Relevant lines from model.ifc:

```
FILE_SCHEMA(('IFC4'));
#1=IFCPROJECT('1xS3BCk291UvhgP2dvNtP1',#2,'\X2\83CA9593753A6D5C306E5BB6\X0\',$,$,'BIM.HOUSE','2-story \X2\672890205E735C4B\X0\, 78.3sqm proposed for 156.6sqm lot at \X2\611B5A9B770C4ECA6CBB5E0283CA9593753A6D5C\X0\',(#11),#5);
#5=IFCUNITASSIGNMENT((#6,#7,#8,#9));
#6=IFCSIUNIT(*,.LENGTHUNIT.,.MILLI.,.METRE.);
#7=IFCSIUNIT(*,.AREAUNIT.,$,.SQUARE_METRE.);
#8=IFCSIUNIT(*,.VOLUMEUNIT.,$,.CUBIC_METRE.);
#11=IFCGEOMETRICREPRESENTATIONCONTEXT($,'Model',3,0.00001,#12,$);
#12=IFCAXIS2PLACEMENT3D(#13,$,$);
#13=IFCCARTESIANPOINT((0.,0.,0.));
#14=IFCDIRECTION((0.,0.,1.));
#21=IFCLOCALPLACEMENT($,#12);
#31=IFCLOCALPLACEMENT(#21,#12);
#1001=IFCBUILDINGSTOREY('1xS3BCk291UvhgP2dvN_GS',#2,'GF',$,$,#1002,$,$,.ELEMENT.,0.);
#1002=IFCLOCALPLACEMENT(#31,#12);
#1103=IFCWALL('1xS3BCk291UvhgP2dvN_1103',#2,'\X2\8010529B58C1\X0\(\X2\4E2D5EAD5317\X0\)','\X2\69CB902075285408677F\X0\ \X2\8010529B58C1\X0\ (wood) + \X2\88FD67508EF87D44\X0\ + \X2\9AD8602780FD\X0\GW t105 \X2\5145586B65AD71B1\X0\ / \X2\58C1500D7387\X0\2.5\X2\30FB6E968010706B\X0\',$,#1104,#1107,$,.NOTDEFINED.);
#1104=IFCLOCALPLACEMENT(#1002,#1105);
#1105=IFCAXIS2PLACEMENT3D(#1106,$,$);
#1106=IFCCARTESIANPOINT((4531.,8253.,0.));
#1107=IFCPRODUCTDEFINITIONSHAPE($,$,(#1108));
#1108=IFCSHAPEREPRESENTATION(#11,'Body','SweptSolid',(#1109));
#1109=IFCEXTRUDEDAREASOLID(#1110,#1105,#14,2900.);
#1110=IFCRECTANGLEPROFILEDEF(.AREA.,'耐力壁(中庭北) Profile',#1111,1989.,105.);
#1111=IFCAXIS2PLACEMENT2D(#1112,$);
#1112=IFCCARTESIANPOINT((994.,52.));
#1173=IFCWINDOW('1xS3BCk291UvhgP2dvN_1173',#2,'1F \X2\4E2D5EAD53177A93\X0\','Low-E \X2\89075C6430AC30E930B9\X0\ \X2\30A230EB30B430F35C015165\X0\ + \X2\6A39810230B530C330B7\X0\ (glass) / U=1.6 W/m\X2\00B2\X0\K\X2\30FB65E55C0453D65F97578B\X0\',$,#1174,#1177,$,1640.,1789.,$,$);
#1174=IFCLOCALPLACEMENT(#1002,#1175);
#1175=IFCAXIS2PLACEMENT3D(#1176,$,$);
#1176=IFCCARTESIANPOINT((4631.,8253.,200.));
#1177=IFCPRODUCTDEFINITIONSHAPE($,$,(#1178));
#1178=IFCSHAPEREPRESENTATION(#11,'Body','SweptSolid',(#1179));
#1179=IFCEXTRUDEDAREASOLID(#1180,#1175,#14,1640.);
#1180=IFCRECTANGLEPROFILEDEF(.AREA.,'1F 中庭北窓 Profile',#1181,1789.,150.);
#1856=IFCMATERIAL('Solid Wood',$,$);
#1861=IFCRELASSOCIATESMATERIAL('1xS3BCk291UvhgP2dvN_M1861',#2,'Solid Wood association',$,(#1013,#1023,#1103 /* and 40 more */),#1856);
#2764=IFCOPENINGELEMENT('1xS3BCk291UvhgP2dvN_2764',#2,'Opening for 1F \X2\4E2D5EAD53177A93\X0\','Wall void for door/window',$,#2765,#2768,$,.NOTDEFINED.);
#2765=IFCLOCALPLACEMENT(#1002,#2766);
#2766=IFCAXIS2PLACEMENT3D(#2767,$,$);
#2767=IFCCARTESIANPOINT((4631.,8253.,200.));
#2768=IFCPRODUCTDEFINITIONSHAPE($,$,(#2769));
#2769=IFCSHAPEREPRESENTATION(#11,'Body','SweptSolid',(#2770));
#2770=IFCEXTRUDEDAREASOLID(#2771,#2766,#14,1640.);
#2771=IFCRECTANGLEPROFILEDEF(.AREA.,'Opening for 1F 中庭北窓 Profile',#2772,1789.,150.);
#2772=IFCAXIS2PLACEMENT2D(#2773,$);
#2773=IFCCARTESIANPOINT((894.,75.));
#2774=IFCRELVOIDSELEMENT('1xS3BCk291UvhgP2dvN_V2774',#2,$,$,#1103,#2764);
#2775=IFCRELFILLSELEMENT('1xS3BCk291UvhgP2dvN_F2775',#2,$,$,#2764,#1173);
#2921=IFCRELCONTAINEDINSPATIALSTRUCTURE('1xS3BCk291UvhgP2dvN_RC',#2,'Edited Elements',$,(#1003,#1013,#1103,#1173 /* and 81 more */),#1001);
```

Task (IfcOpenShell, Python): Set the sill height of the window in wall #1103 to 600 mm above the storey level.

```python
import numpy as np
import ifcopenshell
import ifcopenshell.api.geometry
import ifcopenshell.geom
import ifcopenshell.util.element
import ifcopenshell.util.placement
import ifcopenshell.util.shape
import ifcopenshell.util.unit

model = ifcopenshell.open("model.ifc")
unit_scale = ifcopenshell.util.unit.calculate_unit_scale(model)

window = model.by_guid("1xS3BCk291UvhgP2dvN_1173")
opening = window.FillsVoids[0].RelatingOpeningElement
storey = ifcopenshell.util.element.get_container(window, ifc_class="IfcBuildingStorey")
level = ifcopenshell.util.placement.get_local_placement(storey.ObjectPlacement)[2, 3]

# The opening's origin need not be at the sill, so measure its lowest point.
shape = ifcopenshell.geom.create_shape(ifcopenshell.geom.settings(), opening)
bottom = ifcopenshell.util.shape.get_shape_bottom_elevation(shape, shape.geometry) / unit_scale
dz = level + 600.0 - bottom

shift = np.array([0.0, 0.0, dz])
# The window is not placed relative to its opening, so move both.
for product in (opening, window):
    matrix = ifcopenshell.util.placement.get_local_placement(product.ObjectPlacement)
    matrix[:3, 3] += shift
    ifcopenshell.api.geometry.edit_object_placement(model, product=product, matrix=matrix, is_si=False)

print(f"moved by {dz * unit_scale:+.3f} m")

model.write("model_updated.ifc")
```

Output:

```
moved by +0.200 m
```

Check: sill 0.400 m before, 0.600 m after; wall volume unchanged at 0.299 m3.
